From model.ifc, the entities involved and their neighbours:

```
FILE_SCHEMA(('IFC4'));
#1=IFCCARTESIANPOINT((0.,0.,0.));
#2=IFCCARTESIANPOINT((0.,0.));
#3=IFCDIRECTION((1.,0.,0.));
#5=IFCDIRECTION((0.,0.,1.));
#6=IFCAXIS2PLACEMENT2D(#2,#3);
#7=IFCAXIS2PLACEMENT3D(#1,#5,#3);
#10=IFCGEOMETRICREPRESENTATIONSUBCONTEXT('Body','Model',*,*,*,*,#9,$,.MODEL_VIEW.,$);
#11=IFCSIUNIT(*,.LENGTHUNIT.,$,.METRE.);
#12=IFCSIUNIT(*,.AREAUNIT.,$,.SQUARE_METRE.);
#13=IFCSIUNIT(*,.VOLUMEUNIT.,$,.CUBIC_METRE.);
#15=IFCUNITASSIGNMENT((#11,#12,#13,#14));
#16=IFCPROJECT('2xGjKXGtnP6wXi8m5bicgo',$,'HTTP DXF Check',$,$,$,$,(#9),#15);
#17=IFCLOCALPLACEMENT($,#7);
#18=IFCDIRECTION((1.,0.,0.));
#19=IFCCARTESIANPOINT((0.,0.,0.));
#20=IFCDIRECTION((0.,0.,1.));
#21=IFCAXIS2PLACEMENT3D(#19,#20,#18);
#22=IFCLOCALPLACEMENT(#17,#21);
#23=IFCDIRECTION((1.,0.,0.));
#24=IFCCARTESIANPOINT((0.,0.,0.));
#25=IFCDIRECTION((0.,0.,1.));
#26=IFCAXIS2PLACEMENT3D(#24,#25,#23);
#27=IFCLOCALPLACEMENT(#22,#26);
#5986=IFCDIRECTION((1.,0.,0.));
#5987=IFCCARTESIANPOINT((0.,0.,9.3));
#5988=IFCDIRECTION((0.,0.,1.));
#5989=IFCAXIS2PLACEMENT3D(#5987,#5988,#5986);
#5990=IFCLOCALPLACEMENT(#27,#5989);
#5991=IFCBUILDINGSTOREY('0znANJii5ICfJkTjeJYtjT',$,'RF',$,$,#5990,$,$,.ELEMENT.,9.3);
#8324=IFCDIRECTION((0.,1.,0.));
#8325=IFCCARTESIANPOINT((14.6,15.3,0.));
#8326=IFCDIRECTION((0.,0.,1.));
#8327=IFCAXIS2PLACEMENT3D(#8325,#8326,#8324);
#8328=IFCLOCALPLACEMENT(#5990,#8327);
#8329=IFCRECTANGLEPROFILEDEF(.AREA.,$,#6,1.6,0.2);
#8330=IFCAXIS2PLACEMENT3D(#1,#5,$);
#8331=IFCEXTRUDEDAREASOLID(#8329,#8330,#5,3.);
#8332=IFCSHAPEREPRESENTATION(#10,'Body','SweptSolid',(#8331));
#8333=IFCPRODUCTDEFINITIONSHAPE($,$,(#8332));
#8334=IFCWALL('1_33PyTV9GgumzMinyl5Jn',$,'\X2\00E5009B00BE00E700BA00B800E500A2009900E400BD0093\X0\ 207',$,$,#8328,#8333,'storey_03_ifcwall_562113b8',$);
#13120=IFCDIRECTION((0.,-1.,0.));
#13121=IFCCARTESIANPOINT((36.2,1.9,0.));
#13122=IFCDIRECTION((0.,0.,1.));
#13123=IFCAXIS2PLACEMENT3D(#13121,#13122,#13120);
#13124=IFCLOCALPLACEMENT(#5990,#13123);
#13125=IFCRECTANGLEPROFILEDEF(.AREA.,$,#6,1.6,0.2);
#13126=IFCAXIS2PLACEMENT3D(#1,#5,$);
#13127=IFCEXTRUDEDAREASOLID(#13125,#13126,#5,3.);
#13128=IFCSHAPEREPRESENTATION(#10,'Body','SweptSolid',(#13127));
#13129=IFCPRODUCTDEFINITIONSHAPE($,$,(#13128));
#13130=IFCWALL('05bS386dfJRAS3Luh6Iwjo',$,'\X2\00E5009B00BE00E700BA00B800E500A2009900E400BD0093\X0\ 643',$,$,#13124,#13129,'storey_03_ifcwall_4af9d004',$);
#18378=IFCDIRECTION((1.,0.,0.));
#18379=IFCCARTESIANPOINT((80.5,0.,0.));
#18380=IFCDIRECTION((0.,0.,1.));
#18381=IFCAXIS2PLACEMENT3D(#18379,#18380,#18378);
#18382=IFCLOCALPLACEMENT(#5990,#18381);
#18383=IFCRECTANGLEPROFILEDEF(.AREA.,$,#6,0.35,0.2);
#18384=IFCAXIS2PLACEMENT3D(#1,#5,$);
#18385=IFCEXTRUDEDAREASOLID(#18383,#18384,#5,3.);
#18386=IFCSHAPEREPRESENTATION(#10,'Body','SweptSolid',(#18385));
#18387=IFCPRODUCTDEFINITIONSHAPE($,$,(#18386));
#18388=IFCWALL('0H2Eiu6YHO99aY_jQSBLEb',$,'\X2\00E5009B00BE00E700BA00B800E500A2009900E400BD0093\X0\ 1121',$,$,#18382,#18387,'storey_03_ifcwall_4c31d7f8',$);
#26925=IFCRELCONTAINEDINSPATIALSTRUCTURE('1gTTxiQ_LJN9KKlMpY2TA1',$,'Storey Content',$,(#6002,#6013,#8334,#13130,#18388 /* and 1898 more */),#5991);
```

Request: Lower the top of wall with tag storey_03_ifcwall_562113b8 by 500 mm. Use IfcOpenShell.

```python
import ifcopenshell
import ifcopenshell.geom
import ifcopenshell.util.representation
import ifcopenshell.util.shape

model = ifcopenshell.open("model.ifc")
settings = ifcopenshell.geom.settings()


def volume(element):
    """Net volume in cubic metres, openings subtracted."""
    shape = ifcopenshell.geom.create_shape(settings, element)
    return ifcopenshell.util.shape.get_volume(shape.geometry)


wall = model.by_guid("1_33PyTV9GgumzMinyl5Jn")
before = volume(wall)

body = ifcopenshell.util.representation.get_representation(wall, "Model", "Body")
solid = body.Items[0]
old_height = solid.Depth
solid.Depth -= 0.5
after = volume(wall)

print(f"height {old_height:g} -> {solid.Depth:g}, volume {before:.3f} -> {after:.3f} m3")

model.write("model_rev.ifc")
```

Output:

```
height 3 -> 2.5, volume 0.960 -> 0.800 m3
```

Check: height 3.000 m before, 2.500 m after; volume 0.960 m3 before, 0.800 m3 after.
